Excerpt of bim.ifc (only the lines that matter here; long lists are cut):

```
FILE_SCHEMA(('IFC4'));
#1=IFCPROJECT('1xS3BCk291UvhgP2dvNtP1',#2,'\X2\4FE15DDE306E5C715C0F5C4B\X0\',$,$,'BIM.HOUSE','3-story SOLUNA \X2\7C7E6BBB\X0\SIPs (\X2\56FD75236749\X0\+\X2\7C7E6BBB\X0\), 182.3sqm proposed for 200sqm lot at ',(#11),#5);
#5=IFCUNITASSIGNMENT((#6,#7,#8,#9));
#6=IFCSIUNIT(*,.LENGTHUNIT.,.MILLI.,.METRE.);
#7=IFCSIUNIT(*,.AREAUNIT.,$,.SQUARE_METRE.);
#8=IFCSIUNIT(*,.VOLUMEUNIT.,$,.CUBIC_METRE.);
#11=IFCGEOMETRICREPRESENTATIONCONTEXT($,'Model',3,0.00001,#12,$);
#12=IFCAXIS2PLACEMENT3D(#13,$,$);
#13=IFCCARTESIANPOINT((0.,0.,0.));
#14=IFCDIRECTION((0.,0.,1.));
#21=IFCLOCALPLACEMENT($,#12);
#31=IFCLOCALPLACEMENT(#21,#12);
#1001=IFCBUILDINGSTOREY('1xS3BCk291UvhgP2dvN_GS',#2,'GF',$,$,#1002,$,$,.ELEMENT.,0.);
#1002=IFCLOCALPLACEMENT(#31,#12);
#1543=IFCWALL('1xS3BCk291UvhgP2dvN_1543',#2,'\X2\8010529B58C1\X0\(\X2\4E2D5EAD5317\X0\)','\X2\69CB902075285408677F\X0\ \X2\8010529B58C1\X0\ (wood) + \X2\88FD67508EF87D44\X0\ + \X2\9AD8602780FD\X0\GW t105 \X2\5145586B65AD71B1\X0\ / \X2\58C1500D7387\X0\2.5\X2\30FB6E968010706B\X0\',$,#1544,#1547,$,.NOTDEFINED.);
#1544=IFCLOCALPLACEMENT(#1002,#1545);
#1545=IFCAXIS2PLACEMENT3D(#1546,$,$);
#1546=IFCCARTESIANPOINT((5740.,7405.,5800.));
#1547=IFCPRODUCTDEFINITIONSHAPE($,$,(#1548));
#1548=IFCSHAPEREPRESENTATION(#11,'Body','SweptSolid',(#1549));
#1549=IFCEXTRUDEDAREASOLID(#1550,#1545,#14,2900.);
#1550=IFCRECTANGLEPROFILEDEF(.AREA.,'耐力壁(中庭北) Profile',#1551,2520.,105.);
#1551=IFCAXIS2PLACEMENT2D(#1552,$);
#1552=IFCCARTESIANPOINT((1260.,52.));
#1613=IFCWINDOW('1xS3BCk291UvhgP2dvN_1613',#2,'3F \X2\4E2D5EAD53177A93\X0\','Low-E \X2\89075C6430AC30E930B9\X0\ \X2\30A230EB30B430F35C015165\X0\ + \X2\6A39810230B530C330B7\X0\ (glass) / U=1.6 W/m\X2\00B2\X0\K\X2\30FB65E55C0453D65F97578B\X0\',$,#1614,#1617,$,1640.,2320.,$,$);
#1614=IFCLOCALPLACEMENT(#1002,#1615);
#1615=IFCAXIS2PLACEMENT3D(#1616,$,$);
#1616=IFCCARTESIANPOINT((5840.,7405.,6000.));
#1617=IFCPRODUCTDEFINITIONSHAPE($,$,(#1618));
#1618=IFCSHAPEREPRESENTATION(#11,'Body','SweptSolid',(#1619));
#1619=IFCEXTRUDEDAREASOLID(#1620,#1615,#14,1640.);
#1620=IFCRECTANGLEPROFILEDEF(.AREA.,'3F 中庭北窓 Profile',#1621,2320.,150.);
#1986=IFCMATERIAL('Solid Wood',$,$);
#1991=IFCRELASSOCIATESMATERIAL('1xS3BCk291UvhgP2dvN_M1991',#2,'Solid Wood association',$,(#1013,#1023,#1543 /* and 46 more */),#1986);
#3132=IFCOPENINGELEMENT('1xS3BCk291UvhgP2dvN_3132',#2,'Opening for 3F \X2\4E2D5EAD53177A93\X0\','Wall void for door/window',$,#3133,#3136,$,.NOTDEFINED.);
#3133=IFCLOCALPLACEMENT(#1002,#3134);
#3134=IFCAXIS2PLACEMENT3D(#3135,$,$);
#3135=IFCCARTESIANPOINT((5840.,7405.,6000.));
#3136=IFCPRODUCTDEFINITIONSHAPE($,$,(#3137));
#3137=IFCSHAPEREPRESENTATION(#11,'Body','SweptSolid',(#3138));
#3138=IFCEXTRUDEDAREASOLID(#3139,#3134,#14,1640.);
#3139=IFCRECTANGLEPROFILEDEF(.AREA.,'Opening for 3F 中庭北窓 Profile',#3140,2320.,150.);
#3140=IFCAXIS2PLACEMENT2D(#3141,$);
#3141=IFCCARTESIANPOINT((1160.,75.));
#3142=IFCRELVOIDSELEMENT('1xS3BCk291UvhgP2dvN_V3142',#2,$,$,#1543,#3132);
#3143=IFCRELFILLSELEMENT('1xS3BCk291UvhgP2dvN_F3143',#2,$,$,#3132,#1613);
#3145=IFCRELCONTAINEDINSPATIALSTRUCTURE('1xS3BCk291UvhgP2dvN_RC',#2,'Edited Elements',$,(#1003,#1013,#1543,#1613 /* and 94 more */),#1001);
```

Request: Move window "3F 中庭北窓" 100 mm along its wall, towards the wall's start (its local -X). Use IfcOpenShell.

```python
import ifcopenshell
import ifcopenshell.api.geometry
import ifcopenshell.util.placement

model = ifcopenshell.open("bim.ifc")

window = model.by_guid("1xS3BCk291UvhgP2dvN_1613")
opening = window.FillsVoids[0].RelatingOpeningElement
wall = opening.VoidsElements[0].RelatingBuildingElement

wall_matrix = ifcopenshell.util.placement.get_local_placement(wall.ObjectPlacement)
shift = wall_matrix[:3, 0] * -100.0
before = ifcopenshell.util.placement.get_local_placement(window.ObjectPlacement)[:3, 3].copy()

# The window is not placed relative to its opening, so move both.
for product in (opening, window):
    matrix = ifcopenshell.util.placement.get_local_placement(product.ObjectPlacement)
    matrix[:3, 3] += shift
    ifcopenshell.api.geometry.edit_object_placement(model, product=product, matrix=matrix, is_si=False)

after = ifcopenshell.util.placement.get_local_placement(window.ObjectPlacement)[:3, 3]
print("window moved by", (after - before).round(3) + 0.0)

model.write("bim_v2.ifc")
```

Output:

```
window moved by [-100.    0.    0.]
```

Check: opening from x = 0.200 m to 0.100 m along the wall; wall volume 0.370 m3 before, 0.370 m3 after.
